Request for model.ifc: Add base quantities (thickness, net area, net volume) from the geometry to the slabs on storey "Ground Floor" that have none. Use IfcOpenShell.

First a look at what the model holds.

```python
import ifcopenshell
import ifcopenshell.util.element
import ifcopenshell.util.unit

model = ifcopenshell.open("model.ifc")
print(model.schema)
for unit_type in ("LENGTHUNIT", "AREAUNIT", "VOLUMEUNIT"):
    print(unit_type, ifcopenshell.util.unit.calculate_unit_scale(model, unit_type))
storey = next(s for s in model.by_type("IfcBuildingStorey") if s.Name == "Ground Floor")
slabs = [e for e in ifcopenshell.util.element.get_decomposition(storey) if e.is_a("IfcSlab")]
for e in sorted(slabs, key=lambda e: e.id()):
    print(e.id(), e.is_a(), e.Name, list(ifcopenshell.util.element.get_psets(e, qtos_only=True)), sep=" | ")
```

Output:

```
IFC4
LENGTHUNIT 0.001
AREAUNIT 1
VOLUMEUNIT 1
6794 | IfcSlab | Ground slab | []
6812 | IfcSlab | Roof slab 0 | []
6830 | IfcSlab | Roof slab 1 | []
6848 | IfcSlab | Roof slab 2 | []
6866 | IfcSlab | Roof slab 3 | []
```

```python
import ifcopenshell
import ifcopenshell.api.pset
import ifcopenshell.geom
import ifcopenshell.util.element
import ifcopenshell.util.shape
import ifcopenshell.util.unit

model = ifcopenshell.open("model.ifc")
unit_scale = ifcopenshell.util.unit.calculate_unit_scale(model)
area_scale = ifcopenshell.util.unit.calculate_unit_scale(model, "AREAUNIT")
volume_scale = ifcopenshell.util.unit.calculate_unit_scale(model, "VOLUMEUNIT")
settings = ifcopenshell.geom.settings()

storey = next(s for s in model.by_type("IfcBuildingStorey") if s.Name == "Ground Floor")
slabs = [e for e in ifcopenshell.util.element.get_decomposition(storey) if e.is_a("IfcSlab")]

for e in sorted(slabs, key=lambda e: e.id()):
    if ifcopenshell.util.element.get_psets(e, qtos_only=True, should_inherit=False):
        continue
    # Geometry comes back in metres, in the element's own axes.
    shape = ifcopenshell.geom.create_shape(settings, e)
    values = {
        "Width": ifcopenshell.util.shape.get_z(shape.geometry) / unit_scale,
        "NetArea": ifcopenshell.util.shape.get_footprint_area(shape.geometry) / area_scale,
        "NetVolume": ifcopenshell.util.shape.get_volume(shape.geometry) / volume_scale,
    }
    qto = ifcopenshell.api.pset.add_qto(model, product=e, name="Qto_SlabBaseQuantities")
    ifcopenshell.api.pset.edit_qto(model, qto=qto, properties=values)
    print(e.id(), {k: round(v, 3) for k, v in values.items()})

model.write("model_v2.ifc")
```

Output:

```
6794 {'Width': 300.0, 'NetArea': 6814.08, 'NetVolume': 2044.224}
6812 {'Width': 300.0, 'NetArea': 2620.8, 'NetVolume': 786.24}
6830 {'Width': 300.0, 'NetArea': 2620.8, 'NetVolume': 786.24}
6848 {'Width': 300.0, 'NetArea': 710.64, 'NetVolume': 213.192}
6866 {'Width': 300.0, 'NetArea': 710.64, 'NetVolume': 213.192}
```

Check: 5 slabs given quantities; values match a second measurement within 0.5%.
